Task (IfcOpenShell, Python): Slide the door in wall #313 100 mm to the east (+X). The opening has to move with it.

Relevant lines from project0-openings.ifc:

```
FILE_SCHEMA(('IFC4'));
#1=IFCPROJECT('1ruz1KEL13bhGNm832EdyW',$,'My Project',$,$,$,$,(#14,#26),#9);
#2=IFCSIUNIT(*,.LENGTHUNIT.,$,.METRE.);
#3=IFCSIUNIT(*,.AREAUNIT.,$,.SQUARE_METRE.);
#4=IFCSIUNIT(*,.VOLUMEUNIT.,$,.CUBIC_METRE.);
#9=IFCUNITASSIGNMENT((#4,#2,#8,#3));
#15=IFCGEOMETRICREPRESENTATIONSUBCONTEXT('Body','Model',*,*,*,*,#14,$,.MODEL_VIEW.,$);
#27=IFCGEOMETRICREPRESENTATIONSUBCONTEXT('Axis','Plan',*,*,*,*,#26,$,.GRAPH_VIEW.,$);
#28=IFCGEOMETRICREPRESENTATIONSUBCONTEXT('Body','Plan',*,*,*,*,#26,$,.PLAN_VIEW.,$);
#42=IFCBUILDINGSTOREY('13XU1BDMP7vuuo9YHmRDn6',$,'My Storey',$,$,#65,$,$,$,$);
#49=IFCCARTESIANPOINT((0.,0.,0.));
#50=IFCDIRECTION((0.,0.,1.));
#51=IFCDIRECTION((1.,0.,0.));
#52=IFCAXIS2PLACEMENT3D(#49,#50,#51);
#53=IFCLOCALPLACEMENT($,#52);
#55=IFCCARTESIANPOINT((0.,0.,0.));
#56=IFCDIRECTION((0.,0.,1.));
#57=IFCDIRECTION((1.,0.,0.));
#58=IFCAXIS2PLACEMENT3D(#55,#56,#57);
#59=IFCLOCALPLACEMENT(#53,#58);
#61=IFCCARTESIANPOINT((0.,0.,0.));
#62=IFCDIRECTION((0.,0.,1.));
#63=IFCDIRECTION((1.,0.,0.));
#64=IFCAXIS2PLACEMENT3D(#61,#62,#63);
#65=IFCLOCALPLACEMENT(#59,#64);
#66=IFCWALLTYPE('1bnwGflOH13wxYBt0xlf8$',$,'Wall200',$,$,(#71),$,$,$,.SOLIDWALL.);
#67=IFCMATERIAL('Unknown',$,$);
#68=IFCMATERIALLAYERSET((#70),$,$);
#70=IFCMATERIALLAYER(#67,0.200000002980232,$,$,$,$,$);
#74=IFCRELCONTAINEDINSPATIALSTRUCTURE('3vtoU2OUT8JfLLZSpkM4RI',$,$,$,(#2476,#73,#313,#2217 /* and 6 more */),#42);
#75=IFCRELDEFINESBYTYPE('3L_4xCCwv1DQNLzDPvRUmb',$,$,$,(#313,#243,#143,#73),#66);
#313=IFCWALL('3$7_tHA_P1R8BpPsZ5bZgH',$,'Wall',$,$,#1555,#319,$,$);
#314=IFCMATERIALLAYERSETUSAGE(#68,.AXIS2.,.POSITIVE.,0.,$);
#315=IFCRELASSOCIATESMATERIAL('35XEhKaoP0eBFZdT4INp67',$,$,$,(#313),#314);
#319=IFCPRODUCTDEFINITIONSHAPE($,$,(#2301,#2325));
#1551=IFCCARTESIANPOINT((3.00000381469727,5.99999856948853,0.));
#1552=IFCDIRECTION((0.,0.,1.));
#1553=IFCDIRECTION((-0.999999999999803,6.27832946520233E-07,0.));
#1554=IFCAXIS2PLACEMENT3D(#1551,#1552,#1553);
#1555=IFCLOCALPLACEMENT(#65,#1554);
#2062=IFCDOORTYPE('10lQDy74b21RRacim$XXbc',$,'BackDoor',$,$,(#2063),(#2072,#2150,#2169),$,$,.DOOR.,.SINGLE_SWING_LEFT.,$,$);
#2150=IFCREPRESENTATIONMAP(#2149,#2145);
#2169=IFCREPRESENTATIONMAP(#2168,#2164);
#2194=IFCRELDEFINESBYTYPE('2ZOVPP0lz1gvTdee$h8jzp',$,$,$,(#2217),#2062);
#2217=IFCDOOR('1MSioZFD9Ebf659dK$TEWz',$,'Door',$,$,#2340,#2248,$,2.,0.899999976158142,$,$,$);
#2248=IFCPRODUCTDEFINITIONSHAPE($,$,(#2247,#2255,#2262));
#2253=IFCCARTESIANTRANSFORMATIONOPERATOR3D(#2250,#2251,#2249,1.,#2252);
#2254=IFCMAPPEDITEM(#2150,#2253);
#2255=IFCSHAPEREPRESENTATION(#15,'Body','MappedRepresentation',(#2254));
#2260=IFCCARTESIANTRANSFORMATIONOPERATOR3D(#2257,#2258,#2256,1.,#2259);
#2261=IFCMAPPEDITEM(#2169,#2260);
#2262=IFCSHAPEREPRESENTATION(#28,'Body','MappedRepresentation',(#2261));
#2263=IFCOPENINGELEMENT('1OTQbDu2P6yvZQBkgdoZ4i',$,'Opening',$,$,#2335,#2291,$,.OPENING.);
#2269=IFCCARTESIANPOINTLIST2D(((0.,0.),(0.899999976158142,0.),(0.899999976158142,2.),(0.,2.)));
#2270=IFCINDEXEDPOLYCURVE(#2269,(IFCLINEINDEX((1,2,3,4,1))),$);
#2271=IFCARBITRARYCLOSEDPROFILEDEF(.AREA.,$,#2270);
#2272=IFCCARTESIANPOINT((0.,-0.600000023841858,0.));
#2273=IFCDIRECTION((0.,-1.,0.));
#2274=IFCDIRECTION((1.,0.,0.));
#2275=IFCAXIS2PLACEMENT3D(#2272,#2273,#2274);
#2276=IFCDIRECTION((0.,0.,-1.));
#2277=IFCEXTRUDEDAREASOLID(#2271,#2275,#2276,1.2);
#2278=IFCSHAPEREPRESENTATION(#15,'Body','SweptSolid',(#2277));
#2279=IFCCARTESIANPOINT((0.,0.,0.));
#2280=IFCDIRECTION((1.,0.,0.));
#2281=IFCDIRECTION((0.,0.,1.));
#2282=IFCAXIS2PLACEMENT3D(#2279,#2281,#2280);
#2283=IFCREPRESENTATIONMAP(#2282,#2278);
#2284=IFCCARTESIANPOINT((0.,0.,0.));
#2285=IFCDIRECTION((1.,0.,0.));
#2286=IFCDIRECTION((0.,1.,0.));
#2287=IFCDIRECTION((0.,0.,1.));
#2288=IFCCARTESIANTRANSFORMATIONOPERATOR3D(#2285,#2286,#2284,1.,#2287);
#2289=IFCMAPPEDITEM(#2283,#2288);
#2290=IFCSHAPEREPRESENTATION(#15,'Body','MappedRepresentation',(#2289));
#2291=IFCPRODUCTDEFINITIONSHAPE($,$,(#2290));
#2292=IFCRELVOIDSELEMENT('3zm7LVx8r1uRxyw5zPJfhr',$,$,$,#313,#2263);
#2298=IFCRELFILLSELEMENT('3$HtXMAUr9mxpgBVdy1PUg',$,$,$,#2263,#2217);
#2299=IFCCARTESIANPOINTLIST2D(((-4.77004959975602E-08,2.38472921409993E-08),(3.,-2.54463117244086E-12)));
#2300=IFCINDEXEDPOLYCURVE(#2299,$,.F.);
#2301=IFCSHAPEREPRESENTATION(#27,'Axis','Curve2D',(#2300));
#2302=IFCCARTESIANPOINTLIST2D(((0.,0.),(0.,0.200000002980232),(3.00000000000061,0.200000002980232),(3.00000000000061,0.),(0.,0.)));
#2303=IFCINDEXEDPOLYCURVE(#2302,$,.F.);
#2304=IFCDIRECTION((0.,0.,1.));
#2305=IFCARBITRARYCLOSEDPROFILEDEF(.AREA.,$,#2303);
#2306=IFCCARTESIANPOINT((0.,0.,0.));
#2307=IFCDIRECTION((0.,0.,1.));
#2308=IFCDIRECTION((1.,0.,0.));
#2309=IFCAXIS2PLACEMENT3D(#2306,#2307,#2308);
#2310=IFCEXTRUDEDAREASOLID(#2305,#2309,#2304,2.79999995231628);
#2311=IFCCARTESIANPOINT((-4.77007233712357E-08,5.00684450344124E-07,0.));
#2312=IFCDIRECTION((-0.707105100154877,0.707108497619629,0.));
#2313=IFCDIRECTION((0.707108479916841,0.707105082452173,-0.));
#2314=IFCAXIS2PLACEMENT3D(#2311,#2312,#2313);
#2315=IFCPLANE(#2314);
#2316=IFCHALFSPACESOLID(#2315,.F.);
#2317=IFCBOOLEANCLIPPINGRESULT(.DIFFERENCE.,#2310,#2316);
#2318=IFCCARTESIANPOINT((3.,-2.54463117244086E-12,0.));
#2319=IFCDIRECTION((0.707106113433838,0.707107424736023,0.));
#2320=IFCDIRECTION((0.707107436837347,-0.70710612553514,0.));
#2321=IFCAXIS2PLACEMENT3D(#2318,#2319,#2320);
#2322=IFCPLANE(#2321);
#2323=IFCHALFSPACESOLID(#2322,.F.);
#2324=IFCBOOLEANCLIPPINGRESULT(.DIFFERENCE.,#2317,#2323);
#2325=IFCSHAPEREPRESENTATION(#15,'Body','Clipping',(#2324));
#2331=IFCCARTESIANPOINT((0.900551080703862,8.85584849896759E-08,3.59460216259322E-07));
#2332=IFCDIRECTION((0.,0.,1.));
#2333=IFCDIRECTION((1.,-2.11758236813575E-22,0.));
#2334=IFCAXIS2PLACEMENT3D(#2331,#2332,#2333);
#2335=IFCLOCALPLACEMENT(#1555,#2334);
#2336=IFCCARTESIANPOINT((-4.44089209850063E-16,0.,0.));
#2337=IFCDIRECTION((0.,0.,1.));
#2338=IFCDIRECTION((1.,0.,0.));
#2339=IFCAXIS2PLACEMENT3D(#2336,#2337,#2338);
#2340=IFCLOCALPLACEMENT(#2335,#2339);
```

```python
import ifcopenshell
import ifcopenshell.api.geometry
import ifcopenshell.util.placement

model = ifcopenshell.open("project0-openings.ifc")

door = model.by_guid("1MSioZFD9Ebf659dK$TEWz")
opening = door.FillsVoids[0].RelatingOpeningElement
wall = opening.VoidsElements[0].RelatingBuildingElement

wall_matrix = ifcopenshell.util.placement.get_local_placement(wall.ObjectPlacement)
shift = wall_matrix[:3, 0] * -0.1
before = ifcopenshell.util.placement.get_local_placement(door.ObjectPlacement)[:3, 3].copy()

# The door is placed relative to its opening, so it follows when the opening moves.
matrix = ifcopenshell.util.placement.get_local_placement(opening.ObjectPlacement)
matrix[:3, 3] += shift
ifcopenshell.api.geometry.edit_object_placement(
    model, product=opening, matrix=matrix, is_si=False, should_transform_children=True
)

after = ifcopenshell.util.placement.get_local_placement(door.ObjectPlacement)[:3, 3]
print("door moved by", (after - before).round(3) + 0.0)

model.write("project0-openings_updated.ifc")
```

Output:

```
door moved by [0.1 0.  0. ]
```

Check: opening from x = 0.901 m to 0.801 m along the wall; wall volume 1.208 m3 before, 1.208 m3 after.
